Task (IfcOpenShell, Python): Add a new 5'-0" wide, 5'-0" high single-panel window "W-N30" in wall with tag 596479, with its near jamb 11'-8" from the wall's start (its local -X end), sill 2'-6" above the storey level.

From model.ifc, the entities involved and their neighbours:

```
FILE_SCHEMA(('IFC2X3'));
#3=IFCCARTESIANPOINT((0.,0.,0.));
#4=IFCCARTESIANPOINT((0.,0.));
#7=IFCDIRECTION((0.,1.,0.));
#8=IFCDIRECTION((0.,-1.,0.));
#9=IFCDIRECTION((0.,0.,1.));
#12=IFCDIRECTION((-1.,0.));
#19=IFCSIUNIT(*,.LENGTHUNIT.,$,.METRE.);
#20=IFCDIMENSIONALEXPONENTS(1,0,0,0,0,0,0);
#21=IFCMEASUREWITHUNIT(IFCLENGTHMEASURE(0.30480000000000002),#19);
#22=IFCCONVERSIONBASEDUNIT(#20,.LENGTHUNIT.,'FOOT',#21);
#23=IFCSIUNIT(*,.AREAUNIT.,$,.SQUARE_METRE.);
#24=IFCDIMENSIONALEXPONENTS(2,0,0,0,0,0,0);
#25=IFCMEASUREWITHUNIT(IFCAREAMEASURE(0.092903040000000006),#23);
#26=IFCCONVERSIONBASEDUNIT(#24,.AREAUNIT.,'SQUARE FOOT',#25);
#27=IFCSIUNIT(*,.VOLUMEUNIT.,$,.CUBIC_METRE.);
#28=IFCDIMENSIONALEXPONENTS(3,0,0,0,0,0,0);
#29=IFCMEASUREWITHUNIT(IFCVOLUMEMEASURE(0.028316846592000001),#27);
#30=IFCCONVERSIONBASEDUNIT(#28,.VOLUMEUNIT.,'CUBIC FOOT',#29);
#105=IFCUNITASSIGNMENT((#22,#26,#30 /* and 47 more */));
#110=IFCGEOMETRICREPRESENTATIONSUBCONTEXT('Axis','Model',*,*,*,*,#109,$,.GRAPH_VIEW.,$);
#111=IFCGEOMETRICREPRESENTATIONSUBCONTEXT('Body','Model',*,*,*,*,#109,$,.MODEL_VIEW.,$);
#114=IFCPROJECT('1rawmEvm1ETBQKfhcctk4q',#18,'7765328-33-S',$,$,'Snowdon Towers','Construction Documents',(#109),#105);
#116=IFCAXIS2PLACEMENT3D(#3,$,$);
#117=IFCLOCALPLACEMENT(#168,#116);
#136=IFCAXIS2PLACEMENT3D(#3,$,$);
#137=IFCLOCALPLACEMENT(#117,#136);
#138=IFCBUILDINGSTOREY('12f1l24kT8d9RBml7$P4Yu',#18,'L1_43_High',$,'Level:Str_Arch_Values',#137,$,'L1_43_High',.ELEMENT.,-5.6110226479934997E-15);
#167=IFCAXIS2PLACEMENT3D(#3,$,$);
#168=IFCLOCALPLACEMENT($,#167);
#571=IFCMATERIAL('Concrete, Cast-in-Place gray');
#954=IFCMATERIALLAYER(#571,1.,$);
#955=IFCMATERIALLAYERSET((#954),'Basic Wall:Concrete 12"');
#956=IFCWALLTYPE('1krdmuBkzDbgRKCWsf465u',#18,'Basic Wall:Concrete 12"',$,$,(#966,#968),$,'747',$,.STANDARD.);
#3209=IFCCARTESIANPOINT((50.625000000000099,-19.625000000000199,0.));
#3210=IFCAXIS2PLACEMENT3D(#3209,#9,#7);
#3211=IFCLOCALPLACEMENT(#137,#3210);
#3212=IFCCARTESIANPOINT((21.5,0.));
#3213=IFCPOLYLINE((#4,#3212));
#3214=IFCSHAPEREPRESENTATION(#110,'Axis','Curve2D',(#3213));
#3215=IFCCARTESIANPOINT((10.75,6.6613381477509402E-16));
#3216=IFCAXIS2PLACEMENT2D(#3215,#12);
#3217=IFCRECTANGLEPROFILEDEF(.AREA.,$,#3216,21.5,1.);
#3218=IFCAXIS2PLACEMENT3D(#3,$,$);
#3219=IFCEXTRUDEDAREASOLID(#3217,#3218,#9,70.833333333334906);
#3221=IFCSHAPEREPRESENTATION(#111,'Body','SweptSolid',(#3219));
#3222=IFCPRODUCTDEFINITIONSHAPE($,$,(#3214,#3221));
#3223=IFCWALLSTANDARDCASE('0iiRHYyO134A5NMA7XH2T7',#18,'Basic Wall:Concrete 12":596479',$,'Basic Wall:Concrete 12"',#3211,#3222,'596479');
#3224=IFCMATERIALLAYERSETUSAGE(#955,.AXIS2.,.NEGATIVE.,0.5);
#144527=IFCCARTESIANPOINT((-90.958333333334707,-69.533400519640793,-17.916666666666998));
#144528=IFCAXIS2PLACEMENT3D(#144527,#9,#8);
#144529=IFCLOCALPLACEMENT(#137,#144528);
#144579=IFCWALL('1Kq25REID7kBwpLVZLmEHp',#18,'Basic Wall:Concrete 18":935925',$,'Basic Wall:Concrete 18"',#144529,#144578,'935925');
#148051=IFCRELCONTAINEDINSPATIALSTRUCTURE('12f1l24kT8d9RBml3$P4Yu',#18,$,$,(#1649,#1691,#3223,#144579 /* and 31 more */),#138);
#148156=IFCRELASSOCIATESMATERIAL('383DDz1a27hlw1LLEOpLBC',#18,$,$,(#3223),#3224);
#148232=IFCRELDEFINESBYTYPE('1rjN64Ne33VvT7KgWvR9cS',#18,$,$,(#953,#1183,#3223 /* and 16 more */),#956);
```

```python
import numpy as np
import ifcopenshell
import ifcopenshell.api.feature
import ifcopenshell.api.geometry
import ifcopenshell.api.root
import ifcopenshell.api.spatial
import ifcopenshell.api.type
import ifcopenshell.geom
import ifcopenshell.util.element
import ifcopenshell.util.placement
import ifcopenshell.util.representation
import ifcopenshell.util.shape
import ifcopenshell.util.unit

model = ifcopenshell.open("model.ifc")
unit_scale = ifcopenshell.util.unit.calculate_unit_scale(model)
settings = ifcopenshell.geom.settings()


def volume(element):
    """Net volume in cubic metres, openings subtracted."""
    shape = ifcopenshell.geom.create_shape(settings, element)
    return ifcopenshell.util.shape.get_volume(shape.geometry)


wall = model.by_id(3223)
storey = ifcopenshell.util.element.get_container(wall, ifc_class="IfcBuildingStorey")
context = ifcopenshell.util.representation.get_context(model, "Model", "Body", "MODEL_VIEW")
before = volume(wall)

width, height, from_end, sill = 1.524, 1.524, 3.556, 0.762  # metres

# The wall runs along its own X axis, and the end named is its -X end.
wall_shape = ifcopenshell.geom.create_shape(settings, wall)
x, y, z = ifcopenshell.util.shape.get_vertices(wall_shape.geometry).T
start = x.min() + from_end
face, thickness = float(y.min()), float(y.max() - y.min())
wall_matrix = ifcopenshell.util.placement.get_local_placement(wall.ObjectPlacement)
level = ifcopenshell.util.placement.get_local_placement(storey.ObjectPlacement)[2, 3]


def in_wall(x, y):
    """Placement at x, y metres in the wall's axes, at sill height."""
    matrix = wall_matrix.copy()
    matrix[:, 3] = wall_matrix @ np.array([x / unit_scale, y / unit_scale, 0.0, 1.0])
    matrix[2, 3] = level + sill / unit_scale
    return matrix


# Opening: a box that overshoots both wall faces by 50 mm.
opening = ifcopenshell.api.root.create_entity(model, ifc_class="IfcOpeningElement")
box = ifcopenshell.api.geometry.add_wall_representation(
    model, context=context, length=width, height=height, thickness=thickness + 0.1
)
ifcopenshell.api.geometry.assign_representation(model, product=opening, representation=box)
ifcopenshell.api.geometry.edit_object_placement(model, product=opening, matrix=in_wall(start, face - 0.05), is_si=False)
ifcopenshell.api.feature.add_feature(model, feature=opening, element=wall)

window = ifcopenshell.api.root.create_entity(model, ifc_class="IfcWindow", name="W-N30")
window.OverallWidth, window.OverallHeight = width / unit_scale, height / unit_scale
body = ifcopenshell.api.geometry.add_window_representation(
    model,
    context=context,
    overall_width=window.OverallWidth,
    overall_height=window.OverallHeight,
    partition_type="SINGLE_PANEL",
)
ifcopenshell.api.geometry.assign_representation(model, product=window, representation=body)
ifcopenshell.api.spatial.assign_container(model, products=[window], relating_structure=storey)
fills = ifcopenshell.api.feature.add_filling(model, opening=opening, element=window)
fills.OwnerHistory = window.OwnerHistory  # required in IFC2X3

# IFC2X3 keeps the operation on the window style.
style = ifcopenshell.api.root.create_entity(model, ifc_class="IfcWindowStyle", name="W-N30")
style.OperationType, style.ConstructionType = "SINGLE_PANEL", "NOTDEFINED"
style.ParameterTakesPrecedence = style.Sizeable = False
ifcopenshell.api.type.assign_type(model, related_objects=[window], relating_type=style)

# Centre the window in the wall's thickness.
ifcopenshell.api.geometry.edit_object_placement(model, product=window, matrix=in_wall(start, face), is_si=False)
window_shape = ifcopenshell.geom.create_shape(settings, window)
depth = ifcopenshell.util.shape.get_vertices(window_shape.geometry)[:, 1]
offset = face + thickness / 2 - (depth.min() + depth.max()) / 2
ifcopenshell.api.geometry.edit_object_placement(model, product=window, matrix=in_wall(start, offset), is_si=False)

after = volume(wall)

print(f"wall volume {before:.3f} -> {after:.3f} m3")

model.write("model-out.ifc")
```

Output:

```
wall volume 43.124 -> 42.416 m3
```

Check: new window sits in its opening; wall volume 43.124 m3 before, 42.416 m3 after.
